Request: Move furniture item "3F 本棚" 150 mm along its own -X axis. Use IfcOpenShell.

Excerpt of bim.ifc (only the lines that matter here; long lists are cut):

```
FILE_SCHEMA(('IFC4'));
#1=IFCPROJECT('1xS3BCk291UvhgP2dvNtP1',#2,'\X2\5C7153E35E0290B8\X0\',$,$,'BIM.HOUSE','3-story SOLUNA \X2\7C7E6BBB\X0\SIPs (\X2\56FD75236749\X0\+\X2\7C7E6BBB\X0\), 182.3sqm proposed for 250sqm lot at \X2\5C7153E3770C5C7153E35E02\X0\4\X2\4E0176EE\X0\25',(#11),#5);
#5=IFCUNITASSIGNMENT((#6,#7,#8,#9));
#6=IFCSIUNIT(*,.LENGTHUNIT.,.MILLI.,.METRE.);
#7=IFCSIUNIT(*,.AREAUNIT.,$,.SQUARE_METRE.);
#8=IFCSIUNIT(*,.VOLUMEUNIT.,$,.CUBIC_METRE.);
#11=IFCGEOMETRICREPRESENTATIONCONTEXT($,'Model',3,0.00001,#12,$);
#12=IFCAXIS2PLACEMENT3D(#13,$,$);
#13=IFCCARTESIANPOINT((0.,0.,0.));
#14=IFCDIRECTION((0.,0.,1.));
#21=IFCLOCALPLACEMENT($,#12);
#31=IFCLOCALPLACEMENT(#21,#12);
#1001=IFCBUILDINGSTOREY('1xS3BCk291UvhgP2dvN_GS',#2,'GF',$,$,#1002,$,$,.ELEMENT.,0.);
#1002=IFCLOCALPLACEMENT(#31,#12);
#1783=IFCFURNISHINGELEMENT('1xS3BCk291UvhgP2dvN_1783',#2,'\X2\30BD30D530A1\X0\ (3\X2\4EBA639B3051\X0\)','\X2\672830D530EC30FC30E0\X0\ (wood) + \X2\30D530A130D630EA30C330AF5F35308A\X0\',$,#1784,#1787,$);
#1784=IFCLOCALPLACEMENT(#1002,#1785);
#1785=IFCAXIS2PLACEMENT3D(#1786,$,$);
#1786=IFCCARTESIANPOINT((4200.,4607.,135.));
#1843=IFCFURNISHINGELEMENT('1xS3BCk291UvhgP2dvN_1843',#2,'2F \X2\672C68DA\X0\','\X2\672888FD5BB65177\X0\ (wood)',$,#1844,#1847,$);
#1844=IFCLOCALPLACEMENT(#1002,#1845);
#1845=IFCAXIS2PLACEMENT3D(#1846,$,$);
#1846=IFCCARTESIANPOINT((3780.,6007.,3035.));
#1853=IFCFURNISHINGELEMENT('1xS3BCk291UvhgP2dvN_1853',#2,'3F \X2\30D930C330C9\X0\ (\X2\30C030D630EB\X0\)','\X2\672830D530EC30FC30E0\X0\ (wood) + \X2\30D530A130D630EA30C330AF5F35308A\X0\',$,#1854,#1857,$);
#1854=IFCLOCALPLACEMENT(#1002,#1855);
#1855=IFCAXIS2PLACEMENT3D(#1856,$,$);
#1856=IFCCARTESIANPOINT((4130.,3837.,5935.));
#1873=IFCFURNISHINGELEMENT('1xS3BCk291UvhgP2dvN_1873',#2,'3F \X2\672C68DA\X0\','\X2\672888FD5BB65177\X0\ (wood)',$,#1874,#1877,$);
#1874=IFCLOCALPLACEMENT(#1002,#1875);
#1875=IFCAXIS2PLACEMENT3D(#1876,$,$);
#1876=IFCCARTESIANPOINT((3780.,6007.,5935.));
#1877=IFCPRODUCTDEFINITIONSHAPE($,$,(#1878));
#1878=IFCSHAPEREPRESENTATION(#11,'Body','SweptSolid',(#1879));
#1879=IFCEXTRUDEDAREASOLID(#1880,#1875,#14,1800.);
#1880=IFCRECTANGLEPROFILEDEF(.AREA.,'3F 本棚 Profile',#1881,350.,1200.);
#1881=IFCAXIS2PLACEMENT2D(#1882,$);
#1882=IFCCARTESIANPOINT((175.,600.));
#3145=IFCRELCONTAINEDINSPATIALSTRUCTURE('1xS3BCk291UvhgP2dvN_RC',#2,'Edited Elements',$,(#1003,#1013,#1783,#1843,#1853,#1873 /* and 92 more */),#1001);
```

```python
import ifcopenshell
import ifcopenshell.api.geometry
import ifcopenshell.util.placement
import ifcopenshell.util.unit

model = ifcopenshell.open("bim.ifc")
unit_scale = ifcopenshell.util.unit.calculate_unit_scale(model)

item = model.by_id(1873)
matrix = ifcopenshell.util.placement.get_local_placement(item.ObjectPlacement)
matrix[:3, 3] -= matrix[:3, 0] * 0.15 / unit_scale
ifcopenshell.api.geometry.edit_object_placement(model, product=item, matrix=matrix, is_si=False)

print(ifcopenshell.util.placement.get_local_placement(item.ObjectPlacement).round(3) + 0.0)

model.write("bim-out.ifc")
```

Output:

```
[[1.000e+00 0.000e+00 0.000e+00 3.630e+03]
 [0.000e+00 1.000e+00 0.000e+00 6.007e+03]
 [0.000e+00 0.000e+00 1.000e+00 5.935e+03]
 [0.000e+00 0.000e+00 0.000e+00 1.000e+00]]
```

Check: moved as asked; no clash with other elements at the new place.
